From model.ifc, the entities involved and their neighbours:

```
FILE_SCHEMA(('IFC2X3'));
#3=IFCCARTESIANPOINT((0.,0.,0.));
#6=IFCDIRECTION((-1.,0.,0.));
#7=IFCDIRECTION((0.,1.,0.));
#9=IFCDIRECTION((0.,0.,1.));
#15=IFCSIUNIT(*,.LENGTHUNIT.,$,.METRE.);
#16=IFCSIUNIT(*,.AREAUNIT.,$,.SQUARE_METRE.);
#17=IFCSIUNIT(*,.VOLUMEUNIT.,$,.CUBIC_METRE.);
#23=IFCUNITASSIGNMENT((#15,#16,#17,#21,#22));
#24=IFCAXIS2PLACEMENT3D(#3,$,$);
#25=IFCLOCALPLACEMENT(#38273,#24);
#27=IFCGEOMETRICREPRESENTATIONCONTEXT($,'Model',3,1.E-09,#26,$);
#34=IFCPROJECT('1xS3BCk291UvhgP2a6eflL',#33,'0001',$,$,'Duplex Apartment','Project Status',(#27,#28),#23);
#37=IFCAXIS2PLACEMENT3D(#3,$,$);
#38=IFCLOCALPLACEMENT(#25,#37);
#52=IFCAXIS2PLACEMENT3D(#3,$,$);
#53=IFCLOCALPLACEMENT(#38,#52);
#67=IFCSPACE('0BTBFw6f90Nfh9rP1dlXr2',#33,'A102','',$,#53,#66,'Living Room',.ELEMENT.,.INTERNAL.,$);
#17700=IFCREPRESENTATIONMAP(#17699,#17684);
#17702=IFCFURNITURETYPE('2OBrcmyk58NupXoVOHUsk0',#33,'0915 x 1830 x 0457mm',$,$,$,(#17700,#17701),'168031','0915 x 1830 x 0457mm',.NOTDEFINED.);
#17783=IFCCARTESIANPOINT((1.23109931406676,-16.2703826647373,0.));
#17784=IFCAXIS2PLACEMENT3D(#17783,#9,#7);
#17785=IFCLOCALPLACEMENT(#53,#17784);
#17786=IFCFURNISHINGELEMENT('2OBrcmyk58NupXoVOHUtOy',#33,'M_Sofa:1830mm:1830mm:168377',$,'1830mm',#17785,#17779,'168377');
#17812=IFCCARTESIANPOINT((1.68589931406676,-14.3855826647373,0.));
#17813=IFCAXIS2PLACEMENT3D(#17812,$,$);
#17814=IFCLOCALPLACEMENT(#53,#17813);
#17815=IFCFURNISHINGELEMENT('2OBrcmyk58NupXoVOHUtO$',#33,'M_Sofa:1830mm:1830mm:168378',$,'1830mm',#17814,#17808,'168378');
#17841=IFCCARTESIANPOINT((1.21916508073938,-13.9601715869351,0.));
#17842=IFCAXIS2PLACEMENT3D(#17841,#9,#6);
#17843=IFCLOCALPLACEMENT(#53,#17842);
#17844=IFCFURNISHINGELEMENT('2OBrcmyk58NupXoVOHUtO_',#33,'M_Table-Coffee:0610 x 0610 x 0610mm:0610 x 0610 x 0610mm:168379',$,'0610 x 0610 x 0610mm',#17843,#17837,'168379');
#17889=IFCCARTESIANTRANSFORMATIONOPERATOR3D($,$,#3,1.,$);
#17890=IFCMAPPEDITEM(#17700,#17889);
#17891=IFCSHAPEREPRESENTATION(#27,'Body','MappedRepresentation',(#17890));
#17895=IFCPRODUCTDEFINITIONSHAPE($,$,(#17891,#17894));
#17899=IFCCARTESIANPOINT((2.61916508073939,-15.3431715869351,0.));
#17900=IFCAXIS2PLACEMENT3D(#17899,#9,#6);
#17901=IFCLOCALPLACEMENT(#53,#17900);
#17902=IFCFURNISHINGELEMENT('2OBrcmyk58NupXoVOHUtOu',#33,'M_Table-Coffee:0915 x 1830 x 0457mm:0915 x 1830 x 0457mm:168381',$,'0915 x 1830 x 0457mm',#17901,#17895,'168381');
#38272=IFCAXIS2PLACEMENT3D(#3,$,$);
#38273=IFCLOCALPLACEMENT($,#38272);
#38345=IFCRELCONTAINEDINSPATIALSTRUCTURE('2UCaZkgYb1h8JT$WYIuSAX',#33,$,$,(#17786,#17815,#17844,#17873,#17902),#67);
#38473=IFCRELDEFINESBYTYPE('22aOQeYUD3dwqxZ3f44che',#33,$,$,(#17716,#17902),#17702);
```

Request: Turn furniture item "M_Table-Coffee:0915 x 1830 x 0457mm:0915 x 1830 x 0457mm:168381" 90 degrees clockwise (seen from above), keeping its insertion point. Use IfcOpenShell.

```python
import ifcopenshell
import ifcopenshell.api.geometry
import ifcopenshell.util.placement

model = ifcopenshell.open("model.ifc")

item = model.by_guid("2OBrcmyk58NupXoVOHUtOu")
matrix = ifcopenshell.util.placement.get_local_placement(item.ObjectPlacement)
matrix = matrix @ ifcopenshell.util.placement.rotation(-90, "Z")
ifcopenshell.api.geometry.edit_object_placement(model, product=item, matrix=matrix, is_si=False)

print(ifcopenshell.util.placement.get_local_placement(item.ObjectPlacement).round(3) + 0.0)

model.write("model_v2.ifc")
```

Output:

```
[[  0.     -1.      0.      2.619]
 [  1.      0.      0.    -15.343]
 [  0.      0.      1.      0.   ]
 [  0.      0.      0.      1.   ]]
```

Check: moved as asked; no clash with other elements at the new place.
